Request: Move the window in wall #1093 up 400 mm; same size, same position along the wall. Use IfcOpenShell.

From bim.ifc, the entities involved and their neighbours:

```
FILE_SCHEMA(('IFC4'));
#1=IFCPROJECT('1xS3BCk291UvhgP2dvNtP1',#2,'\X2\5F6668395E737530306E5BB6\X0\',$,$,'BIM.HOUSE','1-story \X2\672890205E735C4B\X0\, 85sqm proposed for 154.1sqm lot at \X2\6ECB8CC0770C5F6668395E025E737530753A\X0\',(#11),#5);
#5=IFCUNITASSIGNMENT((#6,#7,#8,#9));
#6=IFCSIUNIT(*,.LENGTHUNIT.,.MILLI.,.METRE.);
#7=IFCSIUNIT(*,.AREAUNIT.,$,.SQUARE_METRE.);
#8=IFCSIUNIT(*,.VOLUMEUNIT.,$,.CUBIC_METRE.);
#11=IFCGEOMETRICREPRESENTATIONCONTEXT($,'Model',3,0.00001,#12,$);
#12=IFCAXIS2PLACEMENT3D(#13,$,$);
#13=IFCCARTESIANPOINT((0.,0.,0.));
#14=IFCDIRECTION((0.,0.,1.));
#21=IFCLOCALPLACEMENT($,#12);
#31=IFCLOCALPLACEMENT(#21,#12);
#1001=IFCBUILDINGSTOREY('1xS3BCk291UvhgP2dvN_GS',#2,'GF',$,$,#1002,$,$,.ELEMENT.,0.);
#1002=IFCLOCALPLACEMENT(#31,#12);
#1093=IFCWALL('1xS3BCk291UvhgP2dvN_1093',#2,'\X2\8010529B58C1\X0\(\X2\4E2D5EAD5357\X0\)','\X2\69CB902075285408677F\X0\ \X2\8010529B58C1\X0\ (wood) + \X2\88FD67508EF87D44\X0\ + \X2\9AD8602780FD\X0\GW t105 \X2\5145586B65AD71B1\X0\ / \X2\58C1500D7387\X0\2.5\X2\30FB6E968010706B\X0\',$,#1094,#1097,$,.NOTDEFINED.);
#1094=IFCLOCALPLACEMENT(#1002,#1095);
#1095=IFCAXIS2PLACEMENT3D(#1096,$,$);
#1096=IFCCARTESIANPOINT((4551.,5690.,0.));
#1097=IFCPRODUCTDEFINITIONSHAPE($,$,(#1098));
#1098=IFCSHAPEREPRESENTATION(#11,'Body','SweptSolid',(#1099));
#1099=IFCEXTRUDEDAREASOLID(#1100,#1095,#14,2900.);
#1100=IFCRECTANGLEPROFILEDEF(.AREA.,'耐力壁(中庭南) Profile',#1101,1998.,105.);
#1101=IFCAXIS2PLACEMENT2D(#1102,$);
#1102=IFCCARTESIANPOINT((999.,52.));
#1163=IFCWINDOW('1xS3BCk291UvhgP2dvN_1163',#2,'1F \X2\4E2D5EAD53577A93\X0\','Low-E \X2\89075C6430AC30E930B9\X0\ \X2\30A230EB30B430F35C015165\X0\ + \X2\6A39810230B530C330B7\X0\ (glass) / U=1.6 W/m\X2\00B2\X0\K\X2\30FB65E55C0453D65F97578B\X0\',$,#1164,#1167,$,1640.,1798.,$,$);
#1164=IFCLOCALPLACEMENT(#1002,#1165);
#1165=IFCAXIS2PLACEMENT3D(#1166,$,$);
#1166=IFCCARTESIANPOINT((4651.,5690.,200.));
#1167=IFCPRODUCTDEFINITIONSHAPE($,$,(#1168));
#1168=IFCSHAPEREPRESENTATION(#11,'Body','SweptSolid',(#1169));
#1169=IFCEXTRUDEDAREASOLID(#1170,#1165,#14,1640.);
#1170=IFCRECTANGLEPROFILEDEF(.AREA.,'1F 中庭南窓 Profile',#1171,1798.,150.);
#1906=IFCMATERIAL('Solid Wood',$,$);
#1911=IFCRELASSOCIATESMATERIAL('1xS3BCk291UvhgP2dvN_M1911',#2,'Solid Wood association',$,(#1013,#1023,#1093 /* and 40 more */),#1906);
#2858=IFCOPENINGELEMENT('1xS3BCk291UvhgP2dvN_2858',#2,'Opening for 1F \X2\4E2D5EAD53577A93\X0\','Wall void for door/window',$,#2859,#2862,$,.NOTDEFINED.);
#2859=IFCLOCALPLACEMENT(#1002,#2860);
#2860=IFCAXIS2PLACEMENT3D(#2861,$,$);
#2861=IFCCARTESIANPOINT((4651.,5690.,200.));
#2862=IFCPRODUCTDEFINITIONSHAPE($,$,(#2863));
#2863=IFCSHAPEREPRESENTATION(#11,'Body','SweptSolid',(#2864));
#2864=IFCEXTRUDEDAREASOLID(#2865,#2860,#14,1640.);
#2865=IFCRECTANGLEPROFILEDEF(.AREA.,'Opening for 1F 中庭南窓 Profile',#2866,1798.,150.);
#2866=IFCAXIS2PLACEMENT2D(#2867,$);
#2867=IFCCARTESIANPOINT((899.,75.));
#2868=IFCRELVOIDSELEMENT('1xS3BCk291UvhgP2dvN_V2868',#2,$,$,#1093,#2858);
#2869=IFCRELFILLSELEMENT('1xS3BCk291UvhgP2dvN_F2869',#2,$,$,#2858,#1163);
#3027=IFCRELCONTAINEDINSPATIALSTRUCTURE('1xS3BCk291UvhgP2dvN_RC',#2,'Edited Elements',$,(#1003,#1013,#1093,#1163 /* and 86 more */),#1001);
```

```python
import numpy as np
import ifcopenshell
import ifcopenshell.api.geometry
import ifcopenshell.util.placement
import ifcopenshell.util.unit

model = ifcopenshell.open("bim.ifc")
unit_scale = ifcopenshell.util.unit.calculate_unit_scale(model)

window = model.by_id(1163)
opening = window.FillsVoids[0].RelatingOpeningElement
dz = 400.0

shift = np.array([0.0, 0.0, dz])
# The window is not placed relative to its opening, so move both.
for product in (opening, window):
    matrix = ifcopenshell.util.placement.get_local_placement(product.ObjectPlacement)
    matrix[:3, 3] += shift
    ifcopenshell.api.geometry.edit_object_placement(model, product=product, matrix=matrix, is_si=False)

print(f"moved by {dz * unit_scale:+.3f} m")

model.write("bim_v2.ifc")
```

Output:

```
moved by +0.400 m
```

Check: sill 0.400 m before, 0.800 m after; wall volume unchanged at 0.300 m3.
